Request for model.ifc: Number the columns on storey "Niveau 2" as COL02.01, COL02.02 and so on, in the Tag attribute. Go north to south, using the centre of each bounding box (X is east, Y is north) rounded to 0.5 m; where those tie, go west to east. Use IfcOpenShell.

First a look at what the model holds.

```python
import ifcopenshell
import ifcopenshell.util.element
import ifcopenshell.util.placement

model = ifcopenshell.open("model.ifc")
print(model.schema)
storey = next(s for s in model.by_type("IfcBuildingStorey") if s.Name == "Niveau 2")
columns = [e for e in ifcopenshell.util.element.get_decomposition(storey) if e.is_a("IfcColumn")]
for e in sorted(columns, key=lambda e: e.id()):
    origin = ifcopenshell.util.placement.get_local_placement(e.ObjectPlacement)[:3, 3]
    print(e.id(), e.Tag, e.Name, origin.round(2) + 0.0, sep=" | ")
```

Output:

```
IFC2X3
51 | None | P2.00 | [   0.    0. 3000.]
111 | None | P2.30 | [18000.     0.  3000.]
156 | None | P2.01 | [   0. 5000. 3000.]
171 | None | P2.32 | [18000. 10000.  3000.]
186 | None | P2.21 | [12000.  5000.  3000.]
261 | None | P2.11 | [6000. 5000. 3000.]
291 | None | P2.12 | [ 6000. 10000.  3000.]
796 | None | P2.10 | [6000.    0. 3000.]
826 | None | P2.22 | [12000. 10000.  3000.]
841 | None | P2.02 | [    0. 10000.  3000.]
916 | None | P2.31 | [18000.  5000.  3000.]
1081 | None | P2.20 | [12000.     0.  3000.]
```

```python
import ifcopenshell
import ifcopenshell.geom
import ifcopenshell.util.element
import ifcopenshell.util.shape

model = ifcopenshell.open("model.ifc")
settings = ifcopenshell.geom.settings()
settings.set("use-world-coords", True)


def centre(element):
    shape = ifcopenshell.geom.create_shape(settings, element)
    return ifcopenshell.util.shape.get_bbox_centroid(shape.geometry)


storey = next(s for s in model.by_type("IfcBuildingStorey") if s.Name == "Niveau 2")
columns = [e for e in ifcopenshell.util.element.get_decomposition(storey) if e.is_a("IfcColumn")]

# Insertion points can sit at a corner or the storey origin, so sort by the geometry (in metres).
centres = {e: centre(e) for e in columns}
columns.sort(key=lambda e: (-round(centres[e][1] / 0.5), centres[e][0]))

for i, e in enumerate(columns, start=1):
    number = f"COL02.{i:02d}"
    e.Tag = number
    print(e.id(), number)

model.write("model_rev.ifc")
```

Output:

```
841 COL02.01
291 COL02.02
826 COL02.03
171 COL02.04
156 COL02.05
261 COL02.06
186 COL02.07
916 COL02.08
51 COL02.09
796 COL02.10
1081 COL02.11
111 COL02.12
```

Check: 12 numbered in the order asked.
